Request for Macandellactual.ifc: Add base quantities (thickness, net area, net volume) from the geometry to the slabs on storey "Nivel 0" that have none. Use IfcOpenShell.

First a look at what the model holds.

```python
import ifcopenshell
import ifcopenshell.util.element
import ifcopenshell.util.unit

model = ifcopenshell.open("Macandellactual.ifc")
print(model.schema)
for unit_type in ("LENGTHUNIT", "AREAUNIT", "VOLUMEUNIT"):
    print(unit_type, ifcopenshell.util.unit.calculate_unit_scale(model, unit_type))
storey = next(s for s in model.by_type("IfcBuildingStorey") if s.Name == "Nivel 0")
slabs = [e for e in ifcopenshell.util.element.get_decomposition(storey) if e.is_a("IfcSlab")]
for e in sorted(slabs, key=lambda e: e.id()):
    print(e.id(), e.is_a(), e.Name, list(ifcopenshell.util.element.get_psets(e, qtos_only=True)), sep=" | ")
```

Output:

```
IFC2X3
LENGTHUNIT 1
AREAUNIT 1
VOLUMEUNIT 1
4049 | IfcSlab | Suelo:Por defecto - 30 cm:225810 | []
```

```python
import ifcopenshell
import ifcopenshell.api.pset
import ifcopenshell.geom
import ifcopenshell.util.element
import ifcopenshell.util.shape
import ifcopenshell.util.unit

model = ifcopenshell.open("Macandellactual.ifc")
unit_scale = ifcopenshell.util.unit.calculate_unit_scale(model)
area_scale = ifcopenshell.util.unit.calculate_unit_scale(model, "AREAUNIT")
volume_scale = ifcopenshell.util.unit.calculate_unit_scale(model, "VOLUMEUNIT")
settings = ifcopenshell.geom.settings()

storey = next(s for s in model.by_type("IfcBuildingStorey") if s.Name == "Nivel 0")
slabs = [e for e in ifcopenshell.util.element.get_decomposition(storey) if e.is_a("IfcSlab")]

for e in sorted(slabs, key=lambda e: e.id()):
    if ifcopenshell.util.element.get_psets(e, qtos_only=True, should_inherit=False):
        continue
    # Geometry comes back in metres, in the element's own axes.
    shape = ifcopenshell.geom.create_shape(settings, e)
    values = {
        "Width": ifcopenshell.util.shape.get_z(shape.geometry) / unit_scale,
        "NetArea": ifcopenshell.util.shape.get_footprint_area(shape.geometry) / area_scale,
        "NetVolume": ifcopenshell.util.shape.get_volume(shape.geometry) / volume_scale,
    }
    qto = ifcopenshell.api.pset.add_qto(model, product=e, name="BaseQuantities")
    ifcopenshell.api.pset.edit_qto(model, qto=qto, properties=values)
    print(e.id(), {k: round(v, 3) for k, v in values.items()})

model.write("Macandellactual_updated.ifc")
```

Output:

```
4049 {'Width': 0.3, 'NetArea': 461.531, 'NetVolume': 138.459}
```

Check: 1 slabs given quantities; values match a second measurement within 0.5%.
